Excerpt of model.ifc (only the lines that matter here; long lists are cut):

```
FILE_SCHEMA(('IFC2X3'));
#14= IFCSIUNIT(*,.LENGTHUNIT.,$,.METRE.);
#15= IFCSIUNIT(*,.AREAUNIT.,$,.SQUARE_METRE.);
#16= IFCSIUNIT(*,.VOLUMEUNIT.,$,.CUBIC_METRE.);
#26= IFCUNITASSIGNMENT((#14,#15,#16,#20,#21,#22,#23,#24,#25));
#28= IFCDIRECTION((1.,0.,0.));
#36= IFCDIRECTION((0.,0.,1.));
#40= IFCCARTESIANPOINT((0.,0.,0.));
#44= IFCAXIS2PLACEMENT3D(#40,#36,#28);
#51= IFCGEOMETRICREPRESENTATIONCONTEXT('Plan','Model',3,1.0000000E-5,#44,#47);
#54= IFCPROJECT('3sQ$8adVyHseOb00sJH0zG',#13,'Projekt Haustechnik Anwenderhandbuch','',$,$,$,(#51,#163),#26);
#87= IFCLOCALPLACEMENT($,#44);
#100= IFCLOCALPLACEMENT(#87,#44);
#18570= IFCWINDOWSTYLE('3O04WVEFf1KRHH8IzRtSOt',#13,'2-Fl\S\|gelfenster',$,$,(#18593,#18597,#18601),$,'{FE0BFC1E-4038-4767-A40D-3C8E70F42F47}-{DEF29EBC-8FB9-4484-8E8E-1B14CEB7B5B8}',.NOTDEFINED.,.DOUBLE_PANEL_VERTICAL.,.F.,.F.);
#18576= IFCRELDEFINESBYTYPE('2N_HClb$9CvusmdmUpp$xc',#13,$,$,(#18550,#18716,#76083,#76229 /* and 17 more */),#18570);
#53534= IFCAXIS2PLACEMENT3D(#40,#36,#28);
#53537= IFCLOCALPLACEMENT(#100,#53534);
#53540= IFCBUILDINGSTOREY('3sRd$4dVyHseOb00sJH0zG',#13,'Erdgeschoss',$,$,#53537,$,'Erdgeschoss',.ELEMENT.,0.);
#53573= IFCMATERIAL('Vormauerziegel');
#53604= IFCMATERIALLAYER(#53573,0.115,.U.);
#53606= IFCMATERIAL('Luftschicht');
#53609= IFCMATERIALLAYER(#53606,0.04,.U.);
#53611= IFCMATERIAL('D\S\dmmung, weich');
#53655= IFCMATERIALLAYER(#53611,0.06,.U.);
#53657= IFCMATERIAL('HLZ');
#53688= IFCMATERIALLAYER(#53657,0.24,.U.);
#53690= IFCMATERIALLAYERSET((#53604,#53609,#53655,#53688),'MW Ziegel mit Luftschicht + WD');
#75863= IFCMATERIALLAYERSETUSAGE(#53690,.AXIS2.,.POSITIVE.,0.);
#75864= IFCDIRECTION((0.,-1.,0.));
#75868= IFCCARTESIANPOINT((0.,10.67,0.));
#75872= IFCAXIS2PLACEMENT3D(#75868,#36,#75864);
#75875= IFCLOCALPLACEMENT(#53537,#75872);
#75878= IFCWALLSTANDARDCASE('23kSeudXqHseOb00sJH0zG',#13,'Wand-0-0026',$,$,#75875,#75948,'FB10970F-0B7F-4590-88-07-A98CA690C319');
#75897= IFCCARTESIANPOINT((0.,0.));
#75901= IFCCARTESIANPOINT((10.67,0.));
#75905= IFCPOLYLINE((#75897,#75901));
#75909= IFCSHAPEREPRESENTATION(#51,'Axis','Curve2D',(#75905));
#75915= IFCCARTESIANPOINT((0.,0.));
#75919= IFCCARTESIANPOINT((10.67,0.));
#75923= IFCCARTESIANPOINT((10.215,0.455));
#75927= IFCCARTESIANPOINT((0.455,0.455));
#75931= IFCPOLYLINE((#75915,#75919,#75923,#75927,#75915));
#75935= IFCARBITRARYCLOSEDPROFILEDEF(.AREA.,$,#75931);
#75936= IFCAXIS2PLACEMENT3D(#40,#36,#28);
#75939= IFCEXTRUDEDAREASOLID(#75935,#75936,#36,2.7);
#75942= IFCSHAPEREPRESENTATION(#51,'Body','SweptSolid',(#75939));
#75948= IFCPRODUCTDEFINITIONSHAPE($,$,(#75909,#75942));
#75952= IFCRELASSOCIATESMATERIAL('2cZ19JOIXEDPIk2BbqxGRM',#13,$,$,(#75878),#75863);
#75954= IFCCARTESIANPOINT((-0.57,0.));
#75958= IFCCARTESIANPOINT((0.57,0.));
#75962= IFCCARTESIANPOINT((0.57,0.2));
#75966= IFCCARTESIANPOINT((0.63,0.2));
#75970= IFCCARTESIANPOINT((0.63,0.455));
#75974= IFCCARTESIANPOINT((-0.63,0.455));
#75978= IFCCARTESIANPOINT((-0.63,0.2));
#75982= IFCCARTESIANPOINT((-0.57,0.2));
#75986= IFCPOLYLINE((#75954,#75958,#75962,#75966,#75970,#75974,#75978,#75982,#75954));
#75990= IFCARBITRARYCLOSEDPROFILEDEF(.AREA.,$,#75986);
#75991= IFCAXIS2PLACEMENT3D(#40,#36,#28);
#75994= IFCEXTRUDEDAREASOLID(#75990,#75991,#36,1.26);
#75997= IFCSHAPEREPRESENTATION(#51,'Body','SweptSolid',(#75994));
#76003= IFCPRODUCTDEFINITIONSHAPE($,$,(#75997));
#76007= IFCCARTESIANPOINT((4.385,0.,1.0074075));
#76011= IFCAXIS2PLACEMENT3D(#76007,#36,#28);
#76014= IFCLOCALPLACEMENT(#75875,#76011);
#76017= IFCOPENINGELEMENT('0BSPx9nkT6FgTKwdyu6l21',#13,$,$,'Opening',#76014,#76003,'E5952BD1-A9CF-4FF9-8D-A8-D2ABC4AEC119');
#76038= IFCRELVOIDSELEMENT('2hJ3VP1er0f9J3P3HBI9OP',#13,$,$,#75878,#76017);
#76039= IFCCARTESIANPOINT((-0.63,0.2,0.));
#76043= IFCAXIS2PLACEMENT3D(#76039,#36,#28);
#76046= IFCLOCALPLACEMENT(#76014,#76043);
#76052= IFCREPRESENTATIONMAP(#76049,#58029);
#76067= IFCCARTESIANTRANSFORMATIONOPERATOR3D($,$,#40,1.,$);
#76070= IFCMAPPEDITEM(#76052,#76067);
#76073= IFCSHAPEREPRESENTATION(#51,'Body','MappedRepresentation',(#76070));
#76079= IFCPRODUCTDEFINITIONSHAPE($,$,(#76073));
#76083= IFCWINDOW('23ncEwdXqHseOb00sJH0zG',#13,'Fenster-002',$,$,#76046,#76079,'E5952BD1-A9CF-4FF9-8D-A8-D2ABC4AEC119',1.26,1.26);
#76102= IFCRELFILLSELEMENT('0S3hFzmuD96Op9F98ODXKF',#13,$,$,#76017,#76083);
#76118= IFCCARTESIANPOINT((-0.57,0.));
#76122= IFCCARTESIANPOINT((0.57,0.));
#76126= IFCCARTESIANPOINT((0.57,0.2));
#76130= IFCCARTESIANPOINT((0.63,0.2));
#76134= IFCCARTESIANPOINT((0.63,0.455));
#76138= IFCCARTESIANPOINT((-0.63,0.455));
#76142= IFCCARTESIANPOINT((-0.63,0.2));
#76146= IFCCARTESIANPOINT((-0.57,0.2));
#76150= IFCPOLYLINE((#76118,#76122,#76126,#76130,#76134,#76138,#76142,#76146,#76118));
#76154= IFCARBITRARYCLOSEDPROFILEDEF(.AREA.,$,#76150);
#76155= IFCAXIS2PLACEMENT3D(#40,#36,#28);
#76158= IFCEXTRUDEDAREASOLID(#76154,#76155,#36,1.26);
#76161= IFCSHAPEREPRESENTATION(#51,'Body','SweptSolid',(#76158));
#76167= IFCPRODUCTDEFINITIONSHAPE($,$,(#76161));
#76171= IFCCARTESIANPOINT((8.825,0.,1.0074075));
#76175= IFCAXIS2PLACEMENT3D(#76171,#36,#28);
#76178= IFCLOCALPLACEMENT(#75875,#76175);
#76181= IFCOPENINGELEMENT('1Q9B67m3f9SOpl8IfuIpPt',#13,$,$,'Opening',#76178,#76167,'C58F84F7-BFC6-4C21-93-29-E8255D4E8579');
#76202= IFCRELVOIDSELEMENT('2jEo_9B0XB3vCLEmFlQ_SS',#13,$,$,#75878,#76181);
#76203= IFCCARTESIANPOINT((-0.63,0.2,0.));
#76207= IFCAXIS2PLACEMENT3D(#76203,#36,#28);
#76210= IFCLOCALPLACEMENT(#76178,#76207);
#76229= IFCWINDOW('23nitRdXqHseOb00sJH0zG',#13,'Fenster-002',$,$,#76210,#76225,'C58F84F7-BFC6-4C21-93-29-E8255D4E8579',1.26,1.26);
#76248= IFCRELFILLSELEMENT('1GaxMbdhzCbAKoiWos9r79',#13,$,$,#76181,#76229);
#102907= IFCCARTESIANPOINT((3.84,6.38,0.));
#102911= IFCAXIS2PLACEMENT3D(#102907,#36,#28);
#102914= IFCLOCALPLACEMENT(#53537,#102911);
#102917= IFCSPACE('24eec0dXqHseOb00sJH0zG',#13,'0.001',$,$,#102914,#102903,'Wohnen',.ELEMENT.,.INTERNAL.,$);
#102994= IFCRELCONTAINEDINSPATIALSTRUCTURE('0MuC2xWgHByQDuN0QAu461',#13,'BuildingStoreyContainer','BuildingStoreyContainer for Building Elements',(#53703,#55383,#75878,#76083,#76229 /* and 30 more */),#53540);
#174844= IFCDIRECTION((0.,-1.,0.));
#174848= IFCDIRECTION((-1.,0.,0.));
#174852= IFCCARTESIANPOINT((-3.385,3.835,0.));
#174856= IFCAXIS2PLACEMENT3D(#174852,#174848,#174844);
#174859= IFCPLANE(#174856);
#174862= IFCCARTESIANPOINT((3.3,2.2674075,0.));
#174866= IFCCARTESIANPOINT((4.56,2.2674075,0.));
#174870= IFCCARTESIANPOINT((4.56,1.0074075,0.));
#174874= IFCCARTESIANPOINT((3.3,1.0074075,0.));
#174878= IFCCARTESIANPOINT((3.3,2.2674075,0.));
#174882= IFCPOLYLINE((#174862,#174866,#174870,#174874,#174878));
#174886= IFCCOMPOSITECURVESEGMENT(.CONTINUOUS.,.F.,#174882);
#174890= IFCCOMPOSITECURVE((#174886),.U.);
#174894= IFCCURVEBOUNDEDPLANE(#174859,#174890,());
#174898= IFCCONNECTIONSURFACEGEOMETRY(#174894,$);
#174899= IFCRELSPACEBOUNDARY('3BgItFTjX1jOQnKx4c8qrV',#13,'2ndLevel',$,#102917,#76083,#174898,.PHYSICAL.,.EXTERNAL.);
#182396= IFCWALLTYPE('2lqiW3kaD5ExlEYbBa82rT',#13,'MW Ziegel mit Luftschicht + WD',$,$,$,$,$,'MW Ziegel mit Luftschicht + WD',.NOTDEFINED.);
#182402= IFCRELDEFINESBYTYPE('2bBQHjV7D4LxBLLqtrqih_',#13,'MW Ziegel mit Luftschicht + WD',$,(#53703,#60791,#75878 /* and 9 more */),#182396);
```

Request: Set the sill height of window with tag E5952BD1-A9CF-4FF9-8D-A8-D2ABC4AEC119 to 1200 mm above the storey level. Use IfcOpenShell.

```python
import numpy as np
import ifcopenshell
import ifcopenshell.api.geometry
import ifcopenshell.geom
import ifcopenshell.util.element
import ifcopenshell.util.placement
import ifcopenshell.util.shape
import ifcopenshell.util.unit

model = ifcopenshell.open("model.ifc")
unit_scale = ifcopenshell.util.unit.calculate_unit_scale(model)

window = model.by_id(76083)
opening = window.FillsVoids[0].RelatingOpeningElement
storey = ifcopenshell.util.element.get_container(window, ifc_class="IfcBuildingStorey")
level = ifcopenshell.util.placement.get_local_placement(storey.ObjectPlacement)[2, 3]

# The opening's origin need not be at the sill, so measure its lowest point.
shape = ifcopenshell.geom.create_shape(ifcopenshell.geom.settings(), opening)
bottom = ifcopenshell.util.shape.get_shape_bottom_elevation(shape, shape.geometry) / unit_scale
dz = level + 1.2 / unit_scale - bottom

shift = np.array([0.0, 0.0, dz])
# The window is placed relative to its opening, so it follows when the opening moves.
matrix = ifcopenshell.util.placement.get_local_placement(opening.ObjectPlacement)
matrix[:3, 3] += shift
ifcopenshell.api.geometry.edit_object_placement(
    model, product=opening, matrix=matrix, is_si=False, should_transform_children=True
)

# Space boundary surfaces are stored in each space's coordinates; move them too.
for rel in window.ProvidesBoundaries:
    if not rel.ConnectionGeometry:
        continue
    surface = rel.ConnectionGeometry.SurfaceOnRelatingElement.BasisSurface
    space_matrix = ifcopenshell.util.placement.get_local_placement(rel.RelatingSpace.ObjectPlacement)
    point = np.array(surface.Position.Location.Coordinates) + space_matrix[:3, :3].T @ shift
    surface.Position = model.createIfcAxis2Placement3D(
        model.createIfcCartesianPoint(point.tolist()), surface.Position.Axis, surface.Position.RefDirection
    )

print(f"moved by {dz * unit_scale:+.3f} m")

model.write("model_rev.ifc")
```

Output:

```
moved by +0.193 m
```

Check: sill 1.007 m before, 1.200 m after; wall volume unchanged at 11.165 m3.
